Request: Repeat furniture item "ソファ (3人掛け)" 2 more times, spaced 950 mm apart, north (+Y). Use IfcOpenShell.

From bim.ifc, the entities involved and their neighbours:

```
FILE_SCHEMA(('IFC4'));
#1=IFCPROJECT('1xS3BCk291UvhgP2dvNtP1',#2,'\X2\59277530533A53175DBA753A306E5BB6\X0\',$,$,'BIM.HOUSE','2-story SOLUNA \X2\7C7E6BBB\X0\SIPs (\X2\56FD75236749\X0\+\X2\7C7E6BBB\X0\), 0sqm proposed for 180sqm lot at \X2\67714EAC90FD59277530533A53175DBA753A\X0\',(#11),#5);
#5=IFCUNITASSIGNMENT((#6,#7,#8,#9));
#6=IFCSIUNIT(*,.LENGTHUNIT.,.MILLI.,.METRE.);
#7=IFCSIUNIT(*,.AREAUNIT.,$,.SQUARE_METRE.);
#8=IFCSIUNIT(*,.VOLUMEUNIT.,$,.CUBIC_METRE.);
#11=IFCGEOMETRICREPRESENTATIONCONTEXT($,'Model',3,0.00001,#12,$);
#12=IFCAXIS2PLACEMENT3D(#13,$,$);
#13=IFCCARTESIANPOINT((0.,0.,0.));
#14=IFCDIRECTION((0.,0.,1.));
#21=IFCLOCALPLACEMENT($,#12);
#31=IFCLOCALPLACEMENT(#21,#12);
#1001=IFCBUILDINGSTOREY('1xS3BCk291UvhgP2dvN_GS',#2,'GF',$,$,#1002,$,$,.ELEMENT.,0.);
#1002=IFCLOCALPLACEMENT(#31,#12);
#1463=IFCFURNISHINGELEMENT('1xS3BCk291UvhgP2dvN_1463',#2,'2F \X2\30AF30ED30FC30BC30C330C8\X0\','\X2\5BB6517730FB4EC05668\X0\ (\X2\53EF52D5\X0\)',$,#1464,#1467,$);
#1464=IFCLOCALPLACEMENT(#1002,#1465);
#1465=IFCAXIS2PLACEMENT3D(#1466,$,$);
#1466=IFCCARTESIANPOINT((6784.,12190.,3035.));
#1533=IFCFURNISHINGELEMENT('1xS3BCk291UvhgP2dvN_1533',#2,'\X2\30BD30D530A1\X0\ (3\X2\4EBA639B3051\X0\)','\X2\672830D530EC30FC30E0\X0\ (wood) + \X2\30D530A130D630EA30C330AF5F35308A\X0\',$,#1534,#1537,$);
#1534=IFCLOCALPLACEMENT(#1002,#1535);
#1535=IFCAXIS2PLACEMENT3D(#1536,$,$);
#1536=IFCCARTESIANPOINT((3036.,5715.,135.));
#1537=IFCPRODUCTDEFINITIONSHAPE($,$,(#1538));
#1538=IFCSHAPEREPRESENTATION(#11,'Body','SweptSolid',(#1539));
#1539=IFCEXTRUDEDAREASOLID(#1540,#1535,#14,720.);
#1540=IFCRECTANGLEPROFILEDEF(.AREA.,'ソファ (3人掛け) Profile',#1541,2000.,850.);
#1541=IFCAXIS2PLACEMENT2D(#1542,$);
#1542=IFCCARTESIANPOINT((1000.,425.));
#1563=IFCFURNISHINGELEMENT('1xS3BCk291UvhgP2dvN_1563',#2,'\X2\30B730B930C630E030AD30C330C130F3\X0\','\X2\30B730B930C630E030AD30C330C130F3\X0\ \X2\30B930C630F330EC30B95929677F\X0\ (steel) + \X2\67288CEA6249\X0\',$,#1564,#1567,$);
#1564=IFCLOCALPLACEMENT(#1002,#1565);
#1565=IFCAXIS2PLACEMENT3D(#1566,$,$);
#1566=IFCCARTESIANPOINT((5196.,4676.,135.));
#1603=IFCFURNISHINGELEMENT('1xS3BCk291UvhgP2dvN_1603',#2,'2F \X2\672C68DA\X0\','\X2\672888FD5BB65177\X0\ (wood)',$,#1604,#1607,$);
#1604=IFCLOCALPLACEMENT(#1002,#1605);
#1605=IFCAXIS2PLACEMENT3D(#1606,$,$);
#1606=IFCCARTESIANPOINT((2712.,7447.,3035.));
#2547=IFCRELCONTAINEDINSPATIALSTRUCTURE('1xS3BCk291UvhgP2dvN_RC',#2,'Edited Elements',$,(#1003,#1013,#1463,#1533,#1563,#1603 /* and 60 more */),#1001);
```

```python
import numpy as np
import ifcopenshell
import ifcopenshell.api.geometry
import ifcopenshell.api.root
import ifcopenshell.util.element
import ifcopenshell.util.placement
import ifcopenshell.util.unit

model = ifcopenshell.open("bim.ifc")
unit_scale = ifcopenshell.util.unit.calculate_unit_scale(model)


def reuse_history(source, copy):
    """copy_class also copies each property set's owner history, people and application; keep the originals."""
    for rel in copy.IsDefinedBy:
        if rel.is_a("IfcRelDefinesByProperties") and (history := rel.RelatingPropertyDefinition.OwnerHistory):
            rel.RelatingPropertyDefinition.OwnerHistory = source.OwnerHistory
            ifcopenshell.util.element.remove_deep2(model, history)


source = model.by_id(1533)
base = ifcopenshell.util.placement.get_local_placement(source.ObjectPlacement)
step = np.array([0.0, 1.0, 0.0]) * 0.95 / unit_scale

for i in range(1, 3):
    copy = ifcopenshell.api.root.copy_class(model, product=source)
    copy.Representation = ifcopenshell.util.element.copy_deep(
        model, source.Representation, exclude=["IfcGeometricRepresentationContext", "IfcRepresentationMap"]
    )
    reuse_history(source, copy)
    matrix = base.copy()
    matrix[:3, 3] += i * step
    print("added at", matrix[:3, 3].round(3) + 0.0)
    ifcopenshell.api.geometry.edit_object_placement(model, product=copy, matrix=matrix, is_si=False)

model.write("bim_rev.ifc")
```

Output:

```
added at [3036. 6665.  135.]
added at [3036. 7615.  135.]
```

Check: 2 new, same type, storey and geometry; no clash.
